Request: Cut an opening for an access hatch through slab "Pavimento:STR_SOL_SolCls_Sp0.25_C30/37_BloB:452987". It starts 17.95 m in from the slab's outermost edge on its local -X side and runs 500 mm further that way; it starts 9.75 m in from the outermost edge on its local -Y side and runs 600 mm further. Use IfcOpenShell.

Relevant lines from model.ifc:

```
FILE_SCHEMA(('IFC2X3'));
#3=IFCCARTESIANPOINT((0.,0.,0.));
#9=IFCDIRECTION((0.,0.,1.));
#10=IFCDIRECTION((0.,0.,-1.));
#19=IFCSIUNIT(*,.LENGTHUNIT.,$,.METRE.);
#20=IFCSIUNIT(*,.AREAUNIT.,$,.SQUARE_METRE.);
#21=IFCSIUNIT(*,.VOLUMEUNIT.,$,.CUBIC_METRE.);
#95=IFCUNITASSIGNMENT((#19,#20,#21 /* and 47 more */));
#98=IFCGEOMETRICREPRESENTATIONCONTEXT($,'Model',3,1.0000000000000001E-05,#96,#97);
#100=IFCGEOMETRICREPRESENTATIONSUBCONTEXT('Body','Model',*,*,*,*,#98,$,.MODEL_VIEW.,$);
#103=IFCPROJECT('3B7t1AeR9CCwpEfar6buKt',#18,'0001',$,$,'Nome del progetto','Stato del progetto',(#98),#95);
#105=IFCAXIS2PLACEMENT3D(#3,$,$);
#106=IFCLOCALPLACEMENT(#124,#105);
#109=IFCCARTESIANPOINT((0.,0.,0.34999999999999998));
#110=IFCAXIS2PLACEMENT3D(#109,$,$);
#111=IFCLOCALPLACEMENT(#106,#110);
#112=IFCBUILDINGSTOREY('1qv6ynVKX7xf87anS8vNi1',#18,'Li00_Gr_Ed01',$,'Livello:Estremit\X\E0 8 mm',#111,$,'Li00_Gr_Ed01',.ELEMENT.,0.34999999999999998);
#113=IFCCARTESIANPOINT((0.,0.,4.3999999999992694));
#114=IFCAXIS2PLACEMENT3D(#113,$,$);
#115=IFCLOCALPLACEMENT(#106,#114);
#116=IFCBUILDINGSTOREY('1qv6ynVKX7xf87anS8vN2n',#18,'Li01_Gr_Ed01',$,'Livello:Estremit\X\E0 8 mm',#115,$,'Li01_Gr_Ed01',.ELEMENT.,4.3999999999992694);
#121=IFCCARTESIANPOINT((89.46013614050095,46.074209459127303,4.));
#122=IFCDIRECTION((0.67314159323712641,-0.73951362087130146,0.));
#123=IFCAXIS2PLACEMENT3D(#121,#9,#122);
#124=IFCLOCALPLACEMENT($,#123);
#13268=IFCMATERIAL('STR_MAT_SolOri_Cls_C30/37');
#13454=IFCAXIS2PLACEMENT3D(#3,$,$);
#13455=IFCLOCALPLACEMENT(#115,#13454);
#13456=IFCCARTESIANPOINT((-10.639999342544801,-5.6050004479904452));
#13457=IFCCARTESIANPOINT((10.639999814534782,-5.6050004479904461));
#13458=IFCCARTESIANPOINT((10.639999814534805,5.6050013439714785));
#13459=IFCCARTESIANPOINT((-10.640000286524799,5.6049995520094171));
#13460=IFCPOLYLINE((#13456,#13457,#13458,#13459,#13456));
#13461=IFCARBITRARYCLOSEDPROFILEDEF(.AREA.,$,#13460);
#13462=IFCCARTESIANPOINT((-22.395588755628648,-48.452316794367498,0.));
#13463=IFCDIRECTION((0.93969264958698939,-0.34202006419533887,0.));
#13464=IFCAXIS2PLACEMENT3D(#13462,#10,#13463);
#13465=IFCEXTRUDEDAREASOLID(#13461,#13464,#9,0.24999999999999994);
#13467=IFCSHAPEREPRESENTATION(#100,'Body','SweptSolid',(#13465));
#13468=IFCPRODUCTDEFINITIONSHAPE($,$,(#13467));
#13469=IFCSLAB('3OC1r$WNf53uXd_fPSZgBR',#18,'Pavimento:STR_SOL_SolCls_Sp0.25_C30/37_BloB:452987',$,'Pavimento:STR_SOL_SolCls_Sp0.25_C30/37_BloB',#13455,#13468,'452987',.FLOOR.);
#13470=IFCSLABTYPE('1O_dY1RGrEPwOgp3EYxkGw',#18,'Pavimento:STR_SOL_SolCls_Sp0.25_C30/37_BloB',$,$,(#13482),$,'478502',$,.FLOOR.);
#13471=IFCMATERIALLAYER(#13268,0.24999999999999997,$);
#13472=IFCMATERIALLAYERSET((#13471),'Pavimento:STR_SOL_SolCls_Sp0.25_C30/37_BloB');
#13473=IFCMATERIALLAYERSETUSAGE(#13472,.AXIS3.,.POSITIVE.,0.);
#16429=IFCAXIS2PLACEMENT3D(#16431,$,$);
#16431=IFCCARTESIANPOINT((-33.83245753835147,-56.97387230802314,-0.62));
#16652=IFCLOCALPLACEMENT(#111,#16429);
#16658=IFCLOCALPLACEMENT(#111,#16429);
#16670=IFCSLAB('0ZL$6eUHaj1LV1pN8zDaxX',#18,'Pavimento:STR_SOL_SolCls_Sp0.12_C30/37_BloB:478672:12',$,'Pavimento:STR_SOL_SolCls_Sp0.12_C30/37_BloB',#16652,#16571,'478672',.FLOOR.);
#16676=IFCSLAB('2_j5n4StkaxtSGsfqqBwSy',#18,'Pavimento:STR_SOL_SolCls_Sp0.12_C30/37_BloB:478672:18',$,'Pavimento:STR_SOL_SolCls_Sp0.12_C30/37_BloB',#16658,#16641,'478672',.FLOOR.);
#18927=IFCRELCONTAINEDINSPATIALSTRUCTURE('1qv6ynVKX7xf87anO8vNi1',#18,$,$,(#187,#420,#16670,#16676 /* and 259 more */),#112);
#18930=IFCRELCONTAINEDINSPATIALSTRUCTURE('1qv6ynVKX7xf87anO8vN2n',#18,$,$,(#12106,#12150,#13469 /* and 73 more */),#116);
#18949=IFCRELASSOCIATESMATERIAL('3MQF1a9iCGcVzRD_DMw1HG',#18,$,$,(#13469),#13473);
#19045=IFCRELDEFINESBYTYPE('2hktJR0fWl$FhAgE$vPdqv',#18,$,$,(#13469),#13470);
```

```python
import numpy as np
import ifcopenshell
import ifcopenshell.api.feature
import ifcopenshell.api.geometry
import ifcopenshell.api.root
import ifcopenshell.geom
import ifcopenshell.util.placement
import ifcopenshell.util.representation
import ifcopenshell.util.shape
import ifcopenshell.util.unit

model = ifcopenshell.open("model.ifc")
unit_scale = ifcopenshell.util.unit.calculate_unit_scale(model)
settings = ifcopenshell.geom.settings()


def volume(element):
    """Net volume in cubic metres, openings subtracted."""
    shape = ifcopenshell.geom.create_shape(settings, element)
    return ifcopenshell.util.shape.get_volume(shape.geometry)


slab = model.by_guid("3OC1r$WNf53uXd_fPSZgBR")
before = volume(slab)

# Extent in the slab's own axes, in metres. The edges named are its -X and -Y sides.
slab_shape = ifcopenshell.geom.create_shape(settings, slab)
vertices = ifcopenshell.util.shape.get_vertices(slab_shape.geometry)
x_min, y_min, bottom = vertices.min(axis=0)
top = vertices[:, 2].max()

opening = ifcopenshell.api.root.create_entity(model, ifc_class="IfcOpeningElement", name="Access hatch opening")
context = ifcopenshell.util.representation.get_context(model, "Model", "Body", "MODEL_VIEW")
width, depth = 0.5, 0.6
outline = [(0.0, 0.0), (width, 0.0), (width, depth), (0.0, depth), (0.0, 0.0)]
# Overshoot both faces by 50 mm so the cut is clean.
shape = ifcopenshell.api.geometry.add_slab_representation(
    model, context=context, depth=top - bottom + 0.1, polyline=outline
)
ifcopenshell.api.geometry.assign_representation(model, product=opening, representation=shape)

matrix = ifcopenshell.util.placement.get_local_placement(slab.ObjectPlacement)
matrix[:, 3] = matrix @ np.append(np.array([x_min + 17.95, y_min + 9.75, bottom - 0.05]) / unit_scale, 1.0)
ifcopenshell.api.geometry.edit_object_placement(model, product=opening, matrix=matrix, is_si=False)
ifcopenshell.api.feature.add_feature(model, feature=opening, element=slab)

after = volume(slab)

print(f"slab volume {before:.3f} -> {after:.3f} m3")

model.write("model_updated.ifc")
```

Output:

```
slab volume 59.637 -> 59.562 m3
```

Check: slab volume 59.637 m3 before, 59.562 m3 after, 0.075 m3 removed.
